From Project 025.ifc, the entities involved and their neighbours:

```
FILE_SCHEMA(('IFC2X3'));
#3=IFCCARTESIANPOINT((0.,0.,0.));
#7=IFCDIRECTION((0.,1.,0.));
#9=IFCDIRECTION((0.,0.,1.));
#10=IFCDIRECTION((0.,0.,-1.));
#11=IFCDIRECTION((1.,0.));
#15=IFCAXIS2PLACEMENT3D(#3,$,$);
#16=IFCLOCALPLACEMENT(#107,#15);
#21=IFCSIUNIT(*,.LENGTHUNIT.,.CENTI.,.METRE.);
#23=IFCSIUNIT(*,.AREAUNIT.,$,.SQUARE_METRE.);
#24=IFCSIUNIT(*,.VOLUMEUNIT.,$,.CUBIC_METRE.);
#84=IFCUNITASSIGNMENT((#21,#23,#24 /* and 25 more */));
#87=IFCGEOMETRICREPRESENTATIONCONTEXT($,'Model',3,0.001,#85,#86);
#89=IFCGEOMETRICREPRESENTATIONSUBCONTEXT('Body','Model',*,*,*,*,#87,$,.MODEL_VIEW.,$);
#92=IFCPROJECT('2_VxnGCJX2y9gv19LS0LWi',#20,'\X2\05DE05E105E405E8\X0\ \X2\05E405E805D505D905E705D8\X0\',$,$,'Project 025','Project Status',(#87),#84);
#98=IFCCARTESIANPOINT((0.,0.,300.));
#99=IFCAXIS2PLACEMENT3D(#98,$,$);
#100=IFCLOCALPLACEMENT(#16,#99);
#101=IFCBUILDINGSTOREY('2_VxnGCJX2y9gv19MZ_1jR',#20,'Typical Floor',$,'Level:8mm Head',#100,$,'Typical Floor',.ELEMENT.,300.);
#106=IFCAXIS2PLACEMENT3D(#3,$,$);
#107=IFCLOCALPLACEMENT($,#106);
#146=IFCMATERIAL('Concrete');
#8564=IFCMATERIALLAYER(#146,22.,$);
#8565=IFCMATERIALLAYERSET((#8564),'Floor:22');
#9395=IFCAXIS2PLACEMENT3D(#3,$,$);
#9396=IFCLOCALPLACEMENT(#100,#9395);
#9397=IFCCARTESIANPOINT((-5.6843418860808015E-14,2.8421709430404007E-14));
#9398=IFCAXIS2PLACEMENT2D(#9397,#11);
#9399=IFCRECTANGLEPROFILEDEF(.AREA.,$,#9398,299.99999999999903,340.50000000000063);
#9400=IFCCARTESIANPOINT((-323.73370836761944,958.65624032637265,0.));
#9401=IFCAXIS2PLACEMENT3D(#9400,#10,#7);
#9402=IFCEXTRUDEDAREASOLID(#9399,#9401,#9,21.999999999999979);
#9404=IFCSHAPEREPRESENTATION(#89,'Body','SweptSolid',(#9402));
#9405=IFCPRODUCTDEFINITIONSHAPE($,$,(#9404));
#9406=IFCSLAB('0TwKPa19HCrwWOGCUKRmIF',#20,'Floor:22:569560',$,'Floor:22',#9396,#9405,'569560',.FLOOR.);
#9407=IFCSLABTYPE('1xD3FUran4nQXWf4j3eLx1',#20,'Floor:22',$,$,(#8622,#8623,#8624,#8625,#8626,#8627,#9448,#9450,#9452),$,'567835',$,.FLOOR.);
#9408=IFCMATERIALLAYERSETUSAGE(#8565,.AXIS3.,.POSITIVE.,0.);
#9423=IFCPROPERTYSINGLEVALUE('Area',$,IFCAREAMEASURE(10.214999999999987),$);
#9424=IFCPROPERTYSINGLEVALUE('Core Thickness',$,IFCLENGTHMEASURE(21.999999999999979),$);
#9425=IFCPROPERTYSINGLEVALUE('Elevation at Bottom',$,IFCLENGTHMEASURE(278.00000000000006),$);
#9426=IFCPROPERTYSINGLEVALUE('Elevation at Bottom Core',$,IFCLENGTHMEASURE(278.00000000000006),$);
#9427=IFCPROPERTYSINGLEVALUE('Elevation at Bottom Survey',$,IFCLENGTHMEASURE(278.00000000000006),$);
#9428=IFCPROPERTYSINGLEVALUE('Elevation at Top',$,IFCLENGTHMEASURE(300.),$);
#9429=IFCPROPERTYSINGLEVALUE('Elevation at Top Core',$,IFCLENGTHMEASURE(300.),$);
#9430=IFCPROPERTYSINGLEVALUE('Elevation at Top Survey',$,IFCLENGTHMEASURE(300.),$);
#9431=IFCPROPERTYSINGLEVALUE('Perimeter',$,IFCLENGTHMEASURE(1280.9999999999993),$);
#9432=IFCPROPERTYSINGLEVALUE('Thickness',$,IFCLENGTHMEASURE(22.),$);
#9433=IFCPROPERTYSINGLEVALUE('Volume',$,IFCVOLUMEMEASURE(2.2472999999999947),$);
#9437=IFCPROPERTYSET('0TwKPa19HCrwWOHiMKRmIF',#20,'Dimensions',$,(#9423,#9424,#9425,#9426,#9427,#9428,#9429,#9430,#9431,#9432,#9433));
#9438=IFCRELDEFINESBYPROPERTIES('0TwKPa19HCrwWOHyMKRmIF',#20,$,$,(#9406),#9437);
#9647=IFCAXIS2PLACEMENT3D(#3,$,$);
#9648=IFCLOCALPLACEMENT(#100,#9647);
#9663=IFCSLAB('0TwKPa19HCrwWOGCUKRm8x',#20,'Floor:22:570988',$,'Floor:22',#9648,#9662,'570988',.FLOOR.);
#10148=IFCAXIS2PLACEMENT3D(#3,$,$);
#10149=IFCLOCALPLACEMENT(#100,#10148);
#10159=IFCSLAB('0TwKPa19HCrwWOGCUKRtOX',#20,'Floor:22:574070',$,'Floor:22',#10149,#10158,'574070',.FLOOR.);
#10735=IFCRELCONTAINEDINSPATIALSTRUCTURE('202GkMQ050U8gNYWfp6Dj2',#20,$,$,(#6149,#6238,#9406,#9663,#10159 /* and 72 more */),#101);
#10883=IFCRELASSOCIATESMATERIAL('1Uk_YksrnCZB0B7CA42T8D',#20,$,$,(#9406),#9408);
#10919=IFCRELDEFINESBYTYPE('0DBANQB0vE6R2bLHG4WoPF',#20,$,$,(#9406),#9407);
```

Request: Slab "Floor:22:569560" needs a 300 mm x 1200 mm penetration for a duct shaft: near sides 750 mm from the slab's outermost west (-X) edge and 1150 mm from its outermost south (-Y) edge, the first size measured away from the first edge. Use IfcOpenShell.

```python
import numpy as np
import ifcopenshell
import ifcopenshell.api.feature
import ifcopenshell.api.geometry
import ifcopenshell.api.pset
import ifcopenshell.api.root
import ifcopenshell.geom
import ifcopenshell.util.element
import ifcopenshell.util.placement
import ifcopenshell.util.representation
import ifcopenshell.util.shape
import ifcopenshell.util.unit

model = ifcopenshell.open("Project 025.ifc")
unit_scale = ifcopenshell.util.unit.calculate_unit_scale(model)
area_scale = ifcopenshell.util.unit.calculate_unit_scale(model, "AREAUNIT")
volume_scale = ifcopenshell.util.unit.calculate_unit_scale(model, "VOLUMEUNIT")
settings = ifcopenshell.geom.settings()


def volume(element):
    """Net volume in cubic metres, openings subtracted."""
    shape = ifcopenshell.geom.create_shape(settings, element)
    return ifcopenshell.util.shape.get_volume(shape.geometry)


slab = model.by_guid("0TwKPa19HCrwWOGCUKRmIF")
before = volume(slab)

# Extent in the slab's own axes, in metres. The edges named are its -X and -Y sides.
slab_shape = ifcopenshell.geom.create_shape(settings, slab)
vertices = ifcopenshell.util.shape.get_vertices(slab_shape.geometry)
x_min, y_min, bottom = vertices.min(axis=0)
top = vertices[:, 2].max()

opening = ifcopenshell.api.root.create_entity(model, ifc_class="IfcOpeningElement", name="Duct shaft opening")
context = ifcopenshell.util.representation.get_context(model, "Model", "Body", "MODEL_VIEW")
width, depth = 0.3, 1.2
outline = [(0.0, 0.0), (width, 0.0), (width, depth), (0.0, depth), (0.0, 0.0)]
# Overshoot both faces by 50 mm so the cut is clean.
shape = ifcopenshell.api.geometry.add_slab_representation(
    model, context=context, depth=top - bottom + 0.1, polyline=outline
)
ifcopenshell.api.geometry.assign_representation(model, product=opening, representation=shape)

matrix = ifcopenshell.util.placement.get_local_placement(slab.ObjectPlacement)
matrix[:, 3] = matrix @ np.append(np.array([x_min + 0.75, y_min + 1.15, bottom - 0.05]) / unit_scale, 1.0)
ifcopenshell.api.geometry.edit_object_placement(model, product=opening, matrix=matrix, is_si=False)
ifcopenshell.api.feature.add_feature(model, feature=opening, element=slab)

after = volume(slab)

# Update the slab's stored quantities.
pset = model.by_id(ifcopenshell.util.element.get_pset(slab, "Dimensions", should_inherit=False)["id"])
ifcopenshell.api.pset.edit_pset(model, pset=pset, properties={
    "Area": model.create_entity("IfcAreaMeasure", after / (top - bottom) / area_scale),
    "Volume": model.create_entity("IfcVolumeMeasure", after / volume_scale),
})

print(f"slab volume {before:.3f} -> {after:.3f} m3")

model.write("Project 025-out.ifc")
```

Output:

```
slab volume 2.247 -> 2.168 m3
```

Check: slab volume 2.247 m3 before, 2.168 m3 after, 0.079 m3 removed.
